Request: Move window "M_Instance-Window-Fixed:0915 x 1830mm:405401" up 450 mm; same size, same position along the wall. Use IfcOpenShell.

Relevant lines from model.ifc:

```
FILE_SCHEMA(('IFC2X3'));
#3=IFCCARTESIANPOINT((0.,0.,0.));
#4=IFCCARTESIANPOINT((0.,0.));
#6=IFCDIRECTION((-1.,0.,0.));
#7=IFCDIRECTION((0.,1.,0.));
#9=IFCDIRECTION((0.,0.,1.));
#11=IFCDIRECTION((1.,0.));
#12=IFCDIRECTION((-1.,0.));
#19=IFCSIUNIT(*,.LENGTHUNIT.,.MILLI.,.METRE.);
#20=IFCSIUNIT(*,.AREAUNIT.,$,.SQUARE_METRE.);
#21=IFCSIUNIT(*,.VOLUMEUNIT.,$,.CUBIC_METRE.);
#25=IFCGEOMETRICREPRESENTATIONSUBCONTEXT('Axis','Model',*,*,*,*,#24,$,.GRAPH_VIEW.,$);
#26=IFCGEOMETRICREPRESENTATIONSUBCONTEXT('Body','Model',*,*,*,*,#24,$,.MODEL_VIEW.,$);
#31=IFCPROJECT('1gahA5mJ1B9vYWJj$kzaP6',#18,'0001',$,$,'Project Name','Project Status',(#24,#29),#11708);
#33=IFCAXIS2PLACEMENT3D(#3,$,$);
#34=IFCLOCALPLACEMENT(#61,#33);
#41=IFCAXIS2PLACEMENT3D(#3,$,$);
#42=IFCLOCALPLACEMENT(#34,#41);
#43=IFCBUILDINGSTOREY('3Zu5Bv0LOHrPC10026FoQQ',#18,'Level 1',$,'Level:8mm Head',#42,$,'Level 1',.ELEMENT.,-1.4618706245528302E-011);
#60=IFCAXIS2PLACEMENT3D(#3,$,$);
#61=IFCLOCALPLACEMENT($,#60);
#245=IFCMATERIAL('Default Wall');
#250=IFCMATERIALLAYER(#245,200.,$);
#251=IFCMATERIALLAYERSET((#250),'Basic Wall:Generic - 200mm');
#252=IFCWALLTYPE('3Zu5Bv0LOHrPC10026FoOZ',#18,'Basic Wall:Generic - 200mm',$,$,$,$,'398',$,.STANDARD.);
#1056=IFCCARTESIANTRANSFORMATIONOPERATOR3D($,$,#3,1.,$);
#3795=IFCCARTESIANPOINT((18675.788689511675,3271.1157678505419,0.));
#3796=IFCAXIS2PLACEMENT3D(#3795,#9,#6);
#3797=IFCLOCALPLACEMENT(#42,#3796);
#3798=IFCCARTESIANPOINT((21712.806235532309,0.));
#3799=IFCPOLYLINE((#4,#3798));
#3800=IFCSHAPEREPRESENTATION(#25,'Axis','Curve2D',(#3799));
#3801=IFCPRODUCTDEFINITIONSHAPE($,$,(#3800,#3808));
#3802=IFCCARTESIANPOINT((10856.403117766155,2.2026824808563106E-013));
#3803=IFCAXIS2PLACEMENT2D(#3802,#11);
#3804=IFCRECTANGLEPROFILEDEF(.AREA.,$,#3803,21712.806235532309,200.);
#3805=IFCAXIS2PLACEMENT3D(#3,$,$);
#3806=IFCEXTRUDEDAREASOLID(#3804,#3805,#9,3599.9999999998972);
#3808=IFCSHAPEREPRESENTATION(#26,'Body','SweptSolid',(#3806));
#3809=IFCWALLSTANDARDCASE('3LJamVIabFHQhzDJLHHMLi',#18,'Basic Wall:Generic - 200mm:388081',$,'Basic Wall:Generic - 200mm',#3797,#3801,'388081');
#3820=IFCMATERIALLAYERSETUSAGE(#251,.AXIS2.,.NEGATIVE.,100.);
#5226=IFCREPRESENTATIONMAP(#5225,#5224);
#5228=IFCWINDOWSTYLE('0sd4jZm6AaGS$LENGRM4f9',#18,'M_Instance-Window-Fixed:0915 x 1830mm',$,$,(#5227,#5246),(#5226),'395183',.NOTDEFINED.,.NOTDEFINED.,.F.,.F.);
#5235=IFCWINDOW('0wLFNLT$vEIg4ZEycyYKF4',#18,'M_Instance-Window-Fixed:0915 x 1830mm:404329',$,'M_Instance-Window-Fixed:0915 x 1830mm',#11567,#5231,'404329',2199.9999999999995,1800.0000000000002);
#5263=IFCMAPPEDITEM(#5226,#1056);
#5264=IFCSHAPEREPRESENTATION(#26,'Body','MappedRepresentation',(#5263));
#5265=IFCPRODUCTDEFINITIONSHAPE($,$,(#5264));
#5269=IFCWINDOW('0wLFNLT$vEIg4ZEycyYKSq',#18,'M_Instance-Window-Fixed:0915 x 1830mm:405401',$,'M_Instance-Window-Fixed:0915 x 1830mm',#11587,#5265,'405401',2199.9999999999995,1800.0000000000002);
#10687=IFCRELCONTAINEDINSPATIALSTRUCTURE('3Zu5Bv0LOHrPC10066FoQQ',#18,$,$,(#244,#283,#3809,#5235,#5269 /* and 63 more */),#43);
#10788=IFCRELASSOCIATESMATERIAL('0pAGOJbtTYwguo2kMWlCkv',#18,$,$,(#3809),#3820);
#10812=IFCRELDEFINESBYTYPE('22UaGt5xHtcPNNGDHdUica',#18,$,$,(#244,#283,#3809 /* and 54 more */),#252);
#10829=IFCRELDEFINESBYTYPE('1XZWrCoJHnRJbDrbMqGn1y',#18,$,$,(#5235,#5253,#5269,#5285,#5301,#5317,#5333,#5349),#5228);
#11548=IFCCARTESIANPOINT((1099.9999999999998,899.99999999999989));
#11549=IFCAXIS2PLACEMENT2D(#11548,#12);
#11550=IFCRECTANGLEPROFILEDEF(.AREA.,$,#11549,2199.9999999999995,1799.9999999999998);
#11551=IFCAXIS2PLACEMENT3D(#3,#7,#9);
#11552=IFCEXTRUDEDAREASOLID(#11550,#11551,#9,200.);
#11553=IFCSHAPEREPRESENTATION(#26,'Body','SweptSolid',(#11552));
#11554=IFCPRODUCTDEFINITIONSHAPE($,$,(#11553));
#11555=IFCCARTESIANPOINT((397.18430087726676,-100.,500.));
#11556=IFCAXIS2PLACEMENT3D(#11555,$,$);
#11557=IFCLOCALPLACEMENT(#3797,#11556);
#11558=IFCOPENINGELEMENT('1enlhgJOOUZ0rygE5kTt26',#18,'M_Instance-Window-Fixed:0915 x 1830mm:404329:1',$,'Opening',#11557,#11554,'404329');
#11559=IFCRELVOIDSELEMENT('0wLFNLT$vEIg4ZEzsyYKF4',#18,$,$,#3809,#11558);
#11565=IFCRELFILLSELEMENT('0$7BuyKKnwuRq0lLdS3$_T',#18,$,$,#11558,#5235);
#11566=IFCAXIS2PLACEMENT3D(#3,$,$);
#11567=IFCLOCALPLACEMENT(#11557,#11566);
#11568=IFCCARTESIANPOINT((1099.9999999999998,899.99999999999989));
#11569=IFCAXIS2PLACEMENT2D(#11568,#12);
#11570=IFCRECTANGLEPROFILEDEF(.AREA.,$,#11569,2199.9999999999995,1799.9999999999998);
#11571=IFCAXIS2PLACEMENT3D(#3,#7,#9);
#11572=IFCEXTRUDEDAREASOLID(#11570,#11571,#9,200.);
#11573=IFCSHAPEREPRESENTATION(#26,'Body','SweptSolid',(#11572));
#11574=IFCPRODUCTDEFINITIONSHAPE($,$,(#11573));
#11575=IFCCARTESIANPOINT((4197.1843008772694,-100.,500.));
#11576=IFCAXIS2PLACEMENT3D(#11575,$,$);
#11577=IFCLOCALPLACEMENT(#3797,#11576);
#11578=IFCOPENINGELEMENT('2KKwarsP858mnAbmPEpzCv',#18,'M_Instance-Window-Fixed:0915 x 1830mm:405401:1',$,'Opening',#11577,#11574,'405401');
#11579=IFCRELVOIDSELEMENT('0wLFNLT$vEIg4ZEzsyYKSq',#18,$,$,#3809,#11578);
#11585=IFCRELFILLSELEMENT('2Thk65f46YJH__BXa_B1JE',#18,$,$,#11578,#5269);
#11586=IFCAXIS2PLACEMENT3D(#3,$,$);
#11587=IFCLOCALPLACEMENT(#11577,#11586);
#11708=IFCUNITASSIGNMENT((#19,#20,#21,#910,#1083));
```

```python
import numpy as np
import ifcopenshell
import ifcopenshell.api.geometry
import ifcopenshell.util.placement
import ifcopenshell.util.unit

model = ifcopenshell.open("model.ifc")
unit_scale = ifcopenshell.util.unit.calculate_unit_scale(model)

window = model.by_guid("0wLFNLT$vEIg4ZEycyYKSq")
opening = window.FillsVoids[0].RelatingOpeningElement
dz = 450.0

shift = np.array([0.0, 0.0, dz])
# The window is placed relative to its opening, so it follows when the opening moves.
matrix = ifcopenshell.util.placement.get_local_placement(opening.ObjectPlacement)
matrix[:3, 3] += shift
ifcopenshell.api.geometry.edit_object_placement(
    model, product=opening, matrix=matrix, is_si=False, should_transform_children=True
)

print(f"moved by {dz * unit_scale:+.3f} m")

model.write("model_v2.ifc")
```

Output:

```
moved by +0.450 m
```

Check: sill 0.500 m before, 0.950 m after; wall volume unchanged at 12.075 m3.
